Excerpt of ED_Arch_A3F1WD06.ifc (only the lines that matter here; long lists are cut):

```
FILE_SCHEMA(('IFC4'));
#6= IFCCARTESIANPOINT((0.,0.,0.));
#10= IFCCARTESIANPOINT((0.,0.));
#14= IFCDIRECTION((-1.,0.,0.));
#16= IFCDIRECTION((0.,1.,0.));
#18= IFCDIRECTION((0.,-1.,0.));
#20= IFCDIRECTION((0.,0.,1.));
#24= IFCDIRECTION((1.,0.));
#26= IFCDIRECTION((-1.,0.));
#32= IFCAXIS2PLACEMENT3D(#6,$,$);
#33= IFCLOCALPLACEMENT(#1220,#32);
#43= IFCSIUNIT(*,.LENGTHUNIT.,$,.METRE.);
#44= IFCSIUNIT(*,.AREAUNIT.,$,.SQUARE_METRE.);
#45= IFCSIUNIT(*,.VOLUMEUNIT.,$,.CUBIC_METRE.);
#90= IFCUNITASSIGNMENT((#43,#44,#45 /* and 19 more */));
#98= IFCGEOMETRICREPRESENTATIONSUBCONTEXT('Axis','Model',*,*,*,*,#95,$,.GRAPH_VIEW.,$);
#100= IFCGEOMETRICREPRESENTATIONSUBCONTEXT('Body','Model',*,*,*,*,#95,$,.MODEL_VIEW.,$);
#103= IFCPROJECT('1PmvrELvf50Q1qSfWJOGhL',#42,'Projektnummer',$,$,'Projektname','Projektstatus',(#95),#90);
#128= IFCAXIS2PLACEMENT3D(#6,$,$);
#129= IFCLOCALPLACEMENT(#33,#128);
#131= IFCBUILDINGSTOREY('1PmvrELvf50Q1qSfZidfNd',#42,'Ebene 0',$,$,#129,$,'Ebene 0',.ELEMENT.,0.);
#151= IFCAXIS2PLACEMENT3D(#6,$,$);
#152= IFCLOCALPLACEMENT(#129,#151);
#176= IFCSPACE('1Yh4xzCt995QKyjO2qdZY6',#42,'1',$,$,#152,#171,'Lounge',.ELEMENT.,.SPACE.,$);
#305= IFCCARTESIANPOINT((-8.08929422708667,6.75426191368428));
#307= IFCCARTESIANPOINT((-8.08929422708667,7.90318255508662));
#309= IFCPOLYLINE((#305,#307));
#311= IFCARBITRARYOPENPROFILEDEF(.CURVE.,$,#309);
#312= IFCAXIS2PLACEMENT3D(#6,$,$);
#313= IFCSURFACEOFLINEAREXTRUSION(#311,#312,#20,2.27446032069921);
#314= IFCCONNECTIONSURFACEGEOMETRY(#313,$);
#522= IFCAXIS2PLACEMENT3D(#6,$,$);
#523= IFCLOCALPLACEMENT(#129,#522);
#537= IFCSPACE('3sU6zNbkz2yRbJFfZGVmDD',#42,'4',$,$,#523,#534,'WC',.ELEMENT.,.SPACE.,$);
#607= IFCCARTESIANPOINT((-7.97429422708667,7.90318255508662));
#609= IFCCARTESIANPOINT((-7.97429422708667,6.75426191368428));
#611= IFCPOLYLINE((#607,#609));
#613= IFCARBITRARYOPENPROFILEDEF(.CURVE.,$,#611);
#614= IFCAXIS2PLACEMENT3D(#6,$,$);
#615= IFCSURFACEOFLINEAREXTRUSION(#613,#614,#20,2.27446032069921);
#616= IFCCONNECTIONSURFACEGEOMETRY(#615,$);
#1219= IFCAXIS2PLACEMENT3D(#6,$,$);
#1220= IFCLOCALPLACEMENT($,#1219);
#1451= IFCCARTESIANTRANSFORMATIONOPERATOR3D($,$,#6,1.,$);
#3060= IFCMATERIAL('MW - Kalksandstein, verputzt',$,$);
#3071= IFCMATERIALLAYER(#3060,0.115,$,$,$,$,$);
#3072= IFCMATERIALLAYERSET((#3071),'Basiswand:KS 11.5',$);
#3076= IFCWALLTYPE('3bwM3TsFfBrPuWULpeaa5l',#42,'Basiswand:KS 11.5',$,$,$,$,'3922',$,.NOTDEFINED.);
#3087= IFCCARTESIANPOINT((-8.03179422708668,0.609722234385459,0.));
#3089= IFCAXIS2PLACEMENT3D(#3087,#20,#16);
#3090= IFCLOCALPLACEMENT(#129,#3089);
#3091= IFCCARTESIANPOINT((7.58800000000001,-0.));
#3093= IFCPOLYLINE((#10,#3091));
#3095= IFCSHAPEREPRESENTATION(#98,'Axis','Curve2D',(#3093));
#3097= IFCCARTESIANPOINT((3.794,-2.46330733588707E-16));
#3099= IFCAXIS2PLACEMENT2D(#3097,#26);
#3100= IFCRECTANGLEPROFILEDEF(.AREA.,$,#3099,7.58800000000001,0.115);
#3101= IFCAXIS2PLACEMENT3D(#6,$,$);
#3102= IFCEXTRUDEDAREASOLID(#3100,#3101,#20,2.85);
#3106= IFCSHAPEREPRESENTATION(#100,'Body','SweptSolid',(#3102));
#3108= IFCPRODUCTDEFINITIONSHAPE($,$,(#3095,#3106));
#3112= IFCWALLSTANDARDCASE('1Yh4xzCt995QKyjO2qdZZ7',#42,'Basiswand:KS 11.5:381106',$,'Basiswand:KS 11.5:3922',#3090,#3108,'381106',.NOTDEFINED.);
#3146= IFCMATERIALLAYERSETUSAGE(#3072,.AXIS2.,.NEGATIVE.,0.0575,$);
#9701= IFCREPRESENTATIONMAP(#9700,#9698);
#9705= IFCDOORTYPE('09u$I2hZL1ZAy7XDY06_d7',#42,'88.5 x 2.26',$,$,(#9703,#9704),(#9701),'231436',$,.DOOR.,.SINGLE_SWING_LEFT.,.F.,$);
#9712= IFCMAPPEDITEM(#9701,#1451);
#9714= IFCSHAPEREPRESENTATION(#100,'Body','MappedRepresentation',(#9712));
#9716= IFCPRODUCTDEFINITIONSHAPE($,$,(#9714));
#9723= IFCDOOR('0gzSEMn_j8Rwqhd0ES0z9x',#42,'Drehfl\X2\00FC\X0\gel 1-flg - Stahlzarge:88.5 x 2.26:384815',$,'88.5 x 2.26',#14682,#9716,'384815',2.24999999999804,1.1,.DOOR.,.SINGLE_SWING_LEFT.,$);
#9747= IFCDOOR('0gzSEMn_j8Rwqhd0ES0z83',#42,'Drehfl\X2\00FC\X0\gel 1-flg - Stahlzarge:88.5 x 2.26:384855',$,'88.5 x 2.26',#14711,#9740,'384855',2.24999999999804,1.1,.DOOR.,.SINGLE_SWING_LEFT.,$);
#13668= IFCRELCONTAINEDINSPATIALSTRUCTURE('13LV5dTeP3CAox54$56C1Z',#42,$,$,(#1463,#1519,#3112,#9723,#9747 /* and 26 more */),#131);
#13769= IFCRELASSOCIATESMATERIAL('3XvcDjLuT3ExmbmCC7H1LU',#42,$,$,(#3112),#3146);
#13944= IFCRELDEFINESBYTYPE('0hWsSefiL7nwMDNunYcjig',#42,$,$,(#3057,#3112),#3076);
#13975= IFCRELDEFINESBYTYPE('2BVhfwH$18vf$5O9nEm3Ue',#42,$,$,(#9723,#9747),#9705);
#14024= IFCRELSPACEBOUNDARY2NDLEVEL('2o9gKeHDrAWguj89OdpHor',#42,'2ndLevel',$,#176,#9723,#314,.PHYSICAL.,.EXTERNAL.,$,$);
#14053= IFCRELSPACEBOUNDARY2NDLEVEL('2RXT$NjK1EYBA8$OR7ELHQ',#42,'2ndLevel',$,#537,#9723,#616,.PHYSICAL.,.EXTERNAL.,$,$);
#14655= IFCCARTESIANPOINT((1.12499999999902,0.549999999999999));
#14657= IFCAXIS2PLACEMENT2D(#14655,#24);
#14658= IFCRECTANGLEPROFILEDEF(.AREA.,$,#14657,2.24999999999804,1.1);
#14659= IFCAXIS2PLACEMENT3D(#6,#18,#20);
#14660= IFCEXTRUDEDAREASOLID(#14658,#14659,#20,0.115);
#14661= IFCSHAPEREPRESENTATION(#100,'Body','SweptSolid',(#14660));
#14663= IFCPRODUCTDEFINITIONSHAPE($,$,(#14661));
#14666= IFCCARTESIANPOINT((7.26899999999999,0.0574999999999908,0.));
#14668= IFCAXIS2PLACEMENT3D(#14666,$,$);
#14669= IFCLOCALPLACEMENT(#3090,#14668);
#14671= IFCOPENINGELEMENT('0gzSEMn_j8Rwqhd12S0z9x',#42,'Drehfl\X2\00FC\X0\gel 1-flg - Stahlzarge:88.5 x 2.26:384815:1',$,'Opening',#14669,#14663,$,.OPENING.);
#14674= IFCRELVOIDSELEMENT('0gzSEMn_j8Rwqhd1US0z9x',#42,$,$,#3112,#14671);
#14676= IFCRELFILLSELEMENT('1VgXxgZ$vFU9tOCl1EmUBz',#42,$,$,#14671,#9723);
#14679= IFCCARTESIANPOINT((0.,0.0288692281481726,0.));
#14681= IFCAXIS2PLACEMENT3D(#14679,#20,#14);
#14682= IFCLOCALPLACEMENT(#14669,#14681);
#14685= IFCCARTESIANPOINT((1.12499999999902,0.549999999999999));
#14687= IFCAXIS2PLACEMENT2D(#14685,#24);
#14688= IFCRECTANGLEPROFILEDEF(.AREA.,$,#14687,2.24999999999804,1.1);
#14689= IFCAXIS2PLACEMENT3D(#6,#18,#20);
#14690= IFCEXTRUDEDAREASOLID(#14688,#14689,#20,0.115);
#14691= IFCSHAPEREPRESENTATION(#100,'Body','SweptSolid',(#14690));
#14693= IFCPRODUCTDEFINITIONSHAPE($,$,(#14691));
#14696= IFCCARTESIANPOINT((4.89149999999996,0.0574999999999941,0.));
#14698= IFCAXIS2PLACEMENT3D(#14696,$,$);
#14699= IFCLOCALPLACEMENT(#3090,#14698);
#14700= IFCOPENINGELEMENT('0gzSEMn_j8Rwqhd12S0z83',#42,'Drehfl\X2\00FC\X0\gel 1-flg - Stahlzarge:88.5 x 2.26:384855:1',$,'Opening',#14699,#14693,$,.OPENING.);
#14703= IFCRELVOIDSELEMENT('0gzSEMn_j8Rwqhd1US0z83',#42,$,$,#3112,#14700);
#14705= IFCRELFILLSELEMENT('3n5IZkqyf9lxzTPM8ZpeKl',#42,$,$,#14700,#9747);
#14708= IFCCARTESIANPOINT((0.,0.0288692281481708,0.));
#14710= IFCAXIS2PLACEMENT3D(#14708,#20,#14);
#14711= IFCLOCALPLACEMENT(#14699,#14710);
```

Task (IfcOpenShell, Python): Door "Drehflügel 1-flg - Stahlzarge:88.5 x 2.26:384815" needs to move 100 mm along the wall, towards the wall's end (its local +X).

```python
import numpy as np
import ifcopenshell
import ifcopenshell.api.geometry
import ifcopenshell.util.placement
import ifcopenshell.util.unit

model = ifcopenshell.open("ED_Arch_A3F1WD06.ifc")
unit_scale = ifcopenshell.util.unit.calculate_unit_scale(model)

door = model.by_guid("0gzSEMn_j8Rwqhd0ES0z9x")
opening = door.FillsVoids[0].RelatingOpeningElement
wall = opening.VoidsElements[0].RelatingBuildingElement

wall_matrix = ifcopenshell.util.placement.get_local_placement(wall.ObjectPlacement)
shift = wall_matrix[:3, 0] * 0.1 / unit_scale
before = ifcopenshell.util.placement.get_local_placement(door.ObjectPlacement)[:3, 3].copy()

# The door is placed relative to its opening, so it follows when the opening moves.
matrix = ifcopenshell.util.placement.get_local_placement(opening.ObjectPlacement)
matrix[:3, 3] += shift
ifcopenshell.api.geometry.edit_object_placement(
    model, product=opening, matrix=matrix, is_si=False, should_transform_children=True
)

# Space boundary surfaces are stored in each space's coordinates; move them too.
for rel in door.ProvidesBoundaries:
    if not rel.ConnectionGeometry:
        continue
    surface = rel.ConnectionGeometry.SurfaceOnRelatingElement
    space_matrix = ifcopenshell.util.placement.get_local_placement(rel.RelatingSpace.ObjectPlacement)
    point = np.array(surface.Position.Location.Coordinates) + space_matrix[:3, :3].T @ shift
    surface.Position = model.createIfcAxis2Placement3D(
        model.createIfcCartesianPoint(point.tolist()), surface.Position.Axis, surface.Position.RefDirection
    )

after = ifcopenshell.util.placement.get_local_placement(door.ObjectPlacement)[:3, 3]
print("door moved by", (after - before).round(3) + 0.0)

model.write("ED_Arch_A3F1WD06_v2.ifc")
```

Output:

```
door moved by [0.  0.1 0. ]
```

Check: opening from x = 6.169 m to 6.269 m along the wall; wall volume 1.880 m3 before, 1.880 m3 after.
